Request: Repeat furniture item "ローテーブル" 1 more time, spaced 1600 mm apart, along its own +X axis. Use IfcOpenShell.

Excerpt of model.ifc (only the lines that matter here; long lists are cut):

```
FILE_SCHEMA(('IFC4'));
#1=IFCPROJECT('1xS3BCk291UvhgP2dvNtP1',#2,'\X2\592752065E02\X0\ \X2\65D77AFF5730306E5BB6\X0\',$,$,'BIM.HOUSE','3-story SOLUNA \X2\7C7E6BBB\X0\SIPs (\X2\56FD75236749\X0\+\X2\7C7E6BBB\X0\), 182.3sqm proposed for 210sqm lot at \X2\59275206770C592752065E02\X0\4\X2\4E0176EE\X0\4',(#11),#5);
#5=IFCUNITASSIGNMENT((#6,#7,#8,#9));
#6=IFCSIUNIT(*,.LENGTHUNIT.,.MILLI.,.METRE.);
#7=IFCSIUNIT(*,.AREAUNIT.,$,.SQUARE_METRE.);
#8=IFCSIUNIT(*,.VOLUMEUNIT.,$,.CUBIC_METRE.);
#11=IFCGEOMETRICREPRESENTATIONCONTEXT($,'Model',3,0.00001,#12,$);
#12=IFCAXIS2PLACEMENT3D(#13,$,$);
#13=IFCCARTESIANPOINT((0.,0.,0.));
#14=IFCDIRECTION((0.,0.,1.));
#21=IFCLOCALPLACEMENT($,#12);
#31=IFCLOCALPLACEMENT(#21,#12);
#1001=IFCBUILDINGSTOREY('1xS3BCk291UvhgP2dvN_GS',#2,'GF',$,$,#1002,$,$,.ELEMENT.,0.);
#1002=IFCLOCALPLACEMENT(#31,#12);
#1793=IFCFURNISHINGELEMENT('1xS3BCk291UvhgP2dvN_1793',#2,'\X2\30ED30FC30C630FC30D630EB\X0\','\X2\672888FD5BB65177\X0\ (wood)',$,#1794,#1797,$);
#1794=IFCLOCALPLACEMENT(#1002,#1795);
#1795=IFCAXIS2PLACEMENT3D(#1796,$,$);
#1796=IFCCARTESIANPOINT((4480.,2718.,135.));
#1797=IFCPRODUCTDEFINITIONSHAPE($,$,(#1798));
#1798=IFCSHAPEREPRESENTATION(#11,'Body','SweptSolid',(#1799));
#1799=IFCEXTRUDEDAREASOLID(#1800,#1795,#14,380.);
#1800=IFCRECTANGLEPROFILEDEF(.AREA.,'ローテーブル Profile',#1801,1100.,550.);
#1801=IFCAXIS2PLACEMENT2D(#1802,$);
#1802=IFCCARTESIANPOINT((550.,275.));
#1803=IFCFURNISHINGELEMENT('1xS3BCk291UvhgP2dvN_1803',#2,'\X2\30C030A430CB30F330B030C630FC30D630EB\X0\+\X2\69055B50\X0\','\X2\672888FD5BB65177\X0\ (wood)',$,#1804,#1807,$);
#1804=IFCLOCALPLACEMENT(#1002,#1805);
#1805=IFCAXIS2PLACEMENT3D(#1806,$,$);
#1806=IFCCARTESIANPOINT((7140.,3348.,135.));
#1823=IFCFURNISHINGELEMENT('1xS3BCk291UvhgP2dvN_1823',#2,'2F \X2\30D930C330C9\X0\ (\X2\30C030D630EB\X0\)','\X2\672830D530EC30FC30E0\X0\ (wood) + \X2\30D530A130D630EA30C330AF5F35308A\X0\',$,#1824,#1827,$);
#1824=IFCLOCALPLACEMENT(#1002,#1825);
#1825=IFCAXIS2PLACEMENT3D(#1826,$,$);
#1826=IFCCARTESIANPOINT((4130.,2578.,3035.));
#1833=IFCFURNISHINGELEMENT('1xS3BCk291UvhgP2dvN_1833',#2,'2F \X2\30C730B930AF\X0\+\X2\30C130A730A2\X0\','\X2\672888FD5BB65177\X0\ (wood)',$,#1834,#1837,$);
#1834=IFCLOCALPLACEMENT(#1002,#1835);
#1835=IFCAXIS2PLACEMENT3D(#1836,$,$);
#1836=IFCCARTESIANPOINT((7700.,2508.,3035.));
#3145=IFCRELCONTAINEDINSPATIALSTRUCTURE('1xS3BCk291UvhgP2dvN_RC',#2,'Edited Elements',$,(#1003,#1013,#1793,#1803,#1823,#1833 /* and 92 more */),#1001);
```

```python
import ifcopenshell
import ifcopenshell.api.geometry
import ifcopenshell.api.root
import ifcopenshell.util.element
import ifcopenshell.util.placement

model = ifcopenshell.open("model.ifc")


def reuse_history(source, copy):
    """copy_class also copies each property set's owner history, people and application; keep the originals."""
    for rel in copy.IsDefinedBy:
        if rel.is_a("IfcRelDefinesByProperties") and (history := rel.RelatingPropertyDefinition.OwnerHistory):
            rel.RelatingPropertyDefinition.OwnerHistory = source.OwnerHistory
            ifcopenshell.util.element.remove_deep2(model, history)


source = model.by_id(1793)
base = ifcopenshell.util.placement.get_local_placement(source.ObjectPlacement)
step = base[:3, 0] * 1600.0

for i in range(1, 2):
    copy = ifcopenshell.api.root.copy_class(model, product=source)
    copy.Representation = ifcopenshell.util.element.copy_deep(
        model, source.Representation, exclude=["IfcGeometricRepresentationContext", "IfcRepresentationMap"]
    )
    reuse_history(source, copy)
    matrix = base.copy()
    matrix[:3, 3] += i * step
    print("added at", matrix[:3, 3].round(3) + 0.0)
    ifcopenshell.api.geometry.edit_object_placement(model, product=copy, matrix=matrix, is_si=False)

model.write("model_edited.ifc")
```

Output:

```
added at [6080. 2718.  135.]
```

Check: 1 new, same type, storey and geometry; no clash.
